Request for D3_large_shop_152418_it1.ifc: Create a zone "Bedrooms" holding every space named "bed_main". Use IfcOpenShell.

First a look at what the model holds.

```python
import ifcopenshell

model = ifcopenshell.open("D3_large_shop_152418_it1.ifc")
print(model.schema)
seen = {}
for space in model.by_type("IfcSpace"):
    seen[space.LongName] = seen.get(space.LongName, 0) + 1
for name, count in sorted(seen.items(), key=str):
    print(count, "x", name)
print("zones:", [z.Name for z in model.by_type("IfcZone")][:20])
```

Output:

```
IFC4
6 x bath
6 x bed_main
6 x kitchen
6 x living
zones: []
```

```python
import ifcopenshell
import ifcopenshell.api.group
import ifcopenshell.api.root

model = ifcopenshell.open("D3_large_shop_152418_it1.ifc")

names = {"bed_main"}
spaces = [s for s in model.by_type("IfcSpace") if s.LongName in names]

zone = ifcopenshell.api.root.create_entity(model, ifc_class="IfcZone", name="Bedrooms")
ifcopenshell.api.group.assign_group(model, products=spaces, group=zone)
print(len(spaces), "spaces in", zone.Name)

model.write("D3_large_shop_152418_it1_updated.ifc")
```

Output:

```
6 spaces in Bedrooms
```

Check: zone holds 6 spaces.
